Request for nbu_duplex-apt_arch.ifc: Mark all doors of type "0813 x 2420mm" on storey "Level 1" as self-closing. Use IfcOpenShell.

First a look at what the model holds.

```python
import ifcopenshell
import ifcopenshell.util.element

model = ifcopenshell.open("nbu_duplex-apt_arch.ifc")
print(model.schema)
storey = next(s for s in model.by_type("IfcBuildingStorey") if s.Name == "Level 1")
doors = [e for e in ifcopenshell.util.element.get_decomposition(storey) if e.is_a("IfcDoor")]
seen = {}
for e in doors:
    element_type = ifcopenshell.util.element.get_type(e)
    key = (element_type.Name if element_type != e and element_type else None, ifcopenshell.util.element.get_pset(e, "Pset_DoorCommon", "SelfClosing"))
    seen[key] = seen.get(key, 0) + 1
for (name, value), count in sorted(seen.items(), key=str):
    print(count, "x", name, "|", value)
```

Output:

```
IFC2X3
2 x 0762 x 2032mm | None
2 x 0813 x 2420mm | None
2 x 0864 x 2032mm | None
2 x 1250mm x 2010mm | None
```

```python
import ifcopenshell
import ifcopenshell.api.pset
import ifcopenshell.util.element

model = ifcopenshell.open("nbu_duplex-apt_arch.ifc")

storey = next(s for s in model.by_type("IfcBuildingStorey") if s.Name == "Level 1")
doors = [e for e in ifcopenshell.util.element.get_decomposition(storey) if e.is_a("IfcDoor")]

count = 0
for e in doors:
    element_type = ifcopenshell.util.element.get_type(e)
    if element_type in (None, e) or element_type.Name != "0813 x 2420mm":
        continue
    # add_pset returns the element's existing set when there is one.
    pset = ifcopenshell.api.pset.add_pset(model, product=e, name="Pset_DoorCommon")
    ifcopenshell.api.pset.edit_pset(model, pset=pset, properties={"SelfClosing": True})
    count += 1

print(count, "doors updated")

model.write("nbu_duplex-apt_arch_v2.ifc")
```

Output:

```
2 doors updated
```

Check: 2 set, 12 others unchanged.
